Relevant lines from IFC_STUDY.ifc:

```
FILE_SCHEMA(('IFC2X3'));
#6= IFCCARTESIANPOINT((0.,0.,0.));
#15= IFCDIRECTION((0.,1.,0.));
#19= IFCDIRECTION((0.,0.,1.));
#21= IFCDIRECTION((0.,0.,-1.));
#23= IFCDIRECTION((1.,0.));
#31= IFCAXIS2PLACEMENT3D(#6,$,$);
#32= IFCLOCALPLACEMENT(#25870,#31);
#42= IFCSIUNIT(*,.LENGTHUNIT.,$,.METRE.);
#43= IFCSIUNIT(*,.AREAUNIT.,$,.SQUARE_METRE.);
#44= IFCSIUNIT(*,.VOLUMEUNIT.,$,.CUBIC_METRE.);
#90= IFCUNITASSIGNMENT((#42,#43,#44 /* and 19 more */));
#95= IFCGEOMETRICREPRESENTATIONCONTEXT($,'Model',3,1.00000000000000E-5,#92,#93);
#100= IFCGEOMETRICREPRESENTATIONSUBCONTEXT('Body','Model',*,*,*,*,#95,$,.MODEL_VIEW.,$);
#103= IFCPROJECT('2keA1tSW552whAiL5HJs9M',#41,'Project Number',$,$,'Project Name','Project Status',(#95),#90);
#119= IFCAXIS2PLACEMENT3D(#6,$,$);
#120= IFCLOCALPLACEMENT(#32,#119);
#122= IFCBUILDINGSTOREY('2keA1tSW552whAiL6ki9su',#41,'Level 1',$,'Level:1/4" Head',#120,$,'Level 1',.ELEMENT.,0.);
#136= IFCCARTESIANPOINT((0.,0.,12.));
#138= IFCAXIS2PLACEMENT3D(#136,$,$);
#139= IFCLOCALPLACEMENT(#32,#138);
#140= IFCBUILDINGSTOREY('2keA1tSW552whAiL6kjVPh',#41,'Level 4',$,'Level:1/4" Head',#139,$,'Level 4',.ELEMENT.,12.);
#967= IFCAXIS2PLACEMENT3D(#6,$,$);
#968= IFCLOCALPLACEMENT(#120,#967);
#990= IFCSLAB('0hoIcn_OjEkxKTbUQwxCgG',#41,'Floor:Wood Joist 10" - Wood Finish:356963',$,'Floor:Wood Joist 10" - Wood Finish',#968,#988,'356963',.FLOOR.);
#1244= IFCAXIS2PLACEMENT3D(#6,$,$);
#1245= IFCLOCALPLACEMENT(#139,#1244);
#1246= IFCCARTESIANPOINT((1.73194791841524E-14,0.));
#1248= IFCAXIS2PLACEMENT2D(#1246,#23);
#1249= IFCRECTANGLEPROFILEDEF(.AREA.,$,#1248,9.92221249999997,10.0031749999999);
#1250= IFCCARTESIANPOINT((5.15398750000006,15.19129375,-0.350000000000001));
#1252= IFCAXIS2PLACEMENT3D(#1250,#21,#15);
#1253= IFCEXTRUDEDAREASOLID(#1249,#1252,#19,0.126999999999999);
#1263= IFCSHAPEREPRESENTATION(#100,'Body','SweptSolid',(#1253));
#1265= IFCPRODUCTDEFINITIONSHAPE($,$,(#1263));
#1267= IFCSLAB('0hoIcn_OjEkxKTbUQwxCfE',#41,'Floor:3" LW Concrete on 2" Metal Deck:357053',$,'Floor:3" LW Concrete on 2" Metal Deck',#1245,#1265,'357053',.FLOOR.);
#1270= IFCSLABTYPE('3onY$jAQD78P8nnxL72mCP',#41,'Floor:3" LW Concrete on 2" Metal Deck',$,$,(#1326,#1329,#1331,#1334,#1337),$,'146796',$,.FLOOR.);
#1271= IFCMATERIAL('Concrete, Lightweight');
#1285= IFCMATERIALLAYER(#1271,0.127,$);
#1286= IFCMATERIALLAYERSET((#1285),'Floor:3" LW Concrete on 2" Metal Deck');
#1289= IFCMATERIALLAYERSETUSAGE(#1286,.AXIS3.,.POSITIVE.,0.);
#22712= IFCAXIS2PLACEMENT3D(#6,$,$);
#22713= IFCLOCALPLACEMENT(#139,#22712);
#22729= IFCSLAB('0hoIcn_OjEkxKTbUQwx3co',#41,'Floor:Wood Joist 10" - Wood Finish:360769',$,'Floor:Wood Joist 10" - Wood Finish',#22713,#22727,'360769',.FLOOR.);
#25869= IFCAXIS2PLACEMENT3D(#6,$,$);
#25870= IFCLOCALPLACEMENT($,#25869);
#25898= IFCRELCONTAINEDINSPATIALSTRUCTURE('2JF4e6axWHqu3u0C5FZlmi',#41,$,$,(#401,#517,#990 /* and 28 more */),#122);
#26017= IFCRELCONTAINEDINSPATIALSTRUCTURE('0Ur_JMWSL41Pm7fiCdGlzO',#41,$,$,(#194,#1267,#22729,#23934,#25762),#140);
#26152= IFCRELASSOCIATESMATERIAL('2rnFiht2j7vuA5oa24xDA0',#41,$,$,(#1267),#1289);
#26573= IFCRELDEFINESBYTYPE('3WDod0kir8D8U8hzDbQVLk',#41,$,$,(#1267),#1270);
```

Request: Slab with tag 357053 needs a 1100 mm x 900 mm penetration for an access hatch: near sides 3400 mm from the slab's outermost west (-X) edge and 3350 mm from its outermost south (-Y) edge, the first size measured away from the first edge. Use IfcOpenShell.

```python
import numpy as np
import ifcopenshell
import ifcopenshell.api.feature
import ifcopenshell.api.geometry
import ifcopenshell.api.root
import ifcopenshell.geom
import ifcopenshell.util.placement
import ifcopenshell.util.representation
import ifcopenshell.util.shape
import ifcopenshell.util.unit

model = ifcopenshell.open("IFC_STUDY.ifc")
unit_scale = ifcopenshell.util.unit.calculate_unit_scale(model)
settings = ifcopenshell.geom.settings()


def volume(element):
    """Net volume in cubic metres, openings subtracted."""
    shape = ifcopenshell.geom.create_shape(settings, element)
    return ifcopenshell.util.shape.get_volume(shape.geometry)


slab = model.by_guid("0hoIcn_OjEkxKTbUQwxCfE")
before = volume(slab)

# Extent in the slab's own axes, in metres. The edges named are its -X and -Y sides.
slab_shape = ifcopenshell.geom.create_shape(settings, slab)
vertices = ifcopenshell.util.shape.get_vertices(slab_shape.geometry)
x_min, y_min, bottom = vertices.min(axis=0)
top = vertices[:, 2].max()

opening = ifcopenshell.api.root.create_entity(model, ifc_class="IfcOpeningElement", name="Access hatch opening")
context = ifcopenshell.util.representation.get_context(model, "Model", "Body", "MODEL_VIEW")
width, depth = 1.1, 0.9
outline = [(0.0, 0.0), (width, 0.0), (width, depth), (0.0, depth), (0.0, 0.0)]
# Overshoot both faces by 50 mm so the cut is clean.
shape = ifcopenshell.api.geometry.add_slab_representation(
    model, context=context, depth=top - bottom + 0.1, polyline=outline
)
ifcopenshell.api.geometry.assign_representation(model, product=opening, representation=shape)

matrix = ifcopenshell.util.placement.get_local_placement(slab.ObjectPlacement)
matrix[:, 3] = matrix @ np.append(np.array([x_min + 3.4, y_min + 3.35, bottom - 0.05]) / unit_scale, 1.0)
ifcopenshell.api.geometry.edit_object_placement(model, product=opening, matrix=matrix, is_si=False)
ifcopenshell.api.feature.add_feature(model, feature=opening, element=slab)

after = volume(slab)

print(f"slab volume {before:.3f} -> {after:.3f} m3")

model.write("IFC_STUDY_updated.ifc")
```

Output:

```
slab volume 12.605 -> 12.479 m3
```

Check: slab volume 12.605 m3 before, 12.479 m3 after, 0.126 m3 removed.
